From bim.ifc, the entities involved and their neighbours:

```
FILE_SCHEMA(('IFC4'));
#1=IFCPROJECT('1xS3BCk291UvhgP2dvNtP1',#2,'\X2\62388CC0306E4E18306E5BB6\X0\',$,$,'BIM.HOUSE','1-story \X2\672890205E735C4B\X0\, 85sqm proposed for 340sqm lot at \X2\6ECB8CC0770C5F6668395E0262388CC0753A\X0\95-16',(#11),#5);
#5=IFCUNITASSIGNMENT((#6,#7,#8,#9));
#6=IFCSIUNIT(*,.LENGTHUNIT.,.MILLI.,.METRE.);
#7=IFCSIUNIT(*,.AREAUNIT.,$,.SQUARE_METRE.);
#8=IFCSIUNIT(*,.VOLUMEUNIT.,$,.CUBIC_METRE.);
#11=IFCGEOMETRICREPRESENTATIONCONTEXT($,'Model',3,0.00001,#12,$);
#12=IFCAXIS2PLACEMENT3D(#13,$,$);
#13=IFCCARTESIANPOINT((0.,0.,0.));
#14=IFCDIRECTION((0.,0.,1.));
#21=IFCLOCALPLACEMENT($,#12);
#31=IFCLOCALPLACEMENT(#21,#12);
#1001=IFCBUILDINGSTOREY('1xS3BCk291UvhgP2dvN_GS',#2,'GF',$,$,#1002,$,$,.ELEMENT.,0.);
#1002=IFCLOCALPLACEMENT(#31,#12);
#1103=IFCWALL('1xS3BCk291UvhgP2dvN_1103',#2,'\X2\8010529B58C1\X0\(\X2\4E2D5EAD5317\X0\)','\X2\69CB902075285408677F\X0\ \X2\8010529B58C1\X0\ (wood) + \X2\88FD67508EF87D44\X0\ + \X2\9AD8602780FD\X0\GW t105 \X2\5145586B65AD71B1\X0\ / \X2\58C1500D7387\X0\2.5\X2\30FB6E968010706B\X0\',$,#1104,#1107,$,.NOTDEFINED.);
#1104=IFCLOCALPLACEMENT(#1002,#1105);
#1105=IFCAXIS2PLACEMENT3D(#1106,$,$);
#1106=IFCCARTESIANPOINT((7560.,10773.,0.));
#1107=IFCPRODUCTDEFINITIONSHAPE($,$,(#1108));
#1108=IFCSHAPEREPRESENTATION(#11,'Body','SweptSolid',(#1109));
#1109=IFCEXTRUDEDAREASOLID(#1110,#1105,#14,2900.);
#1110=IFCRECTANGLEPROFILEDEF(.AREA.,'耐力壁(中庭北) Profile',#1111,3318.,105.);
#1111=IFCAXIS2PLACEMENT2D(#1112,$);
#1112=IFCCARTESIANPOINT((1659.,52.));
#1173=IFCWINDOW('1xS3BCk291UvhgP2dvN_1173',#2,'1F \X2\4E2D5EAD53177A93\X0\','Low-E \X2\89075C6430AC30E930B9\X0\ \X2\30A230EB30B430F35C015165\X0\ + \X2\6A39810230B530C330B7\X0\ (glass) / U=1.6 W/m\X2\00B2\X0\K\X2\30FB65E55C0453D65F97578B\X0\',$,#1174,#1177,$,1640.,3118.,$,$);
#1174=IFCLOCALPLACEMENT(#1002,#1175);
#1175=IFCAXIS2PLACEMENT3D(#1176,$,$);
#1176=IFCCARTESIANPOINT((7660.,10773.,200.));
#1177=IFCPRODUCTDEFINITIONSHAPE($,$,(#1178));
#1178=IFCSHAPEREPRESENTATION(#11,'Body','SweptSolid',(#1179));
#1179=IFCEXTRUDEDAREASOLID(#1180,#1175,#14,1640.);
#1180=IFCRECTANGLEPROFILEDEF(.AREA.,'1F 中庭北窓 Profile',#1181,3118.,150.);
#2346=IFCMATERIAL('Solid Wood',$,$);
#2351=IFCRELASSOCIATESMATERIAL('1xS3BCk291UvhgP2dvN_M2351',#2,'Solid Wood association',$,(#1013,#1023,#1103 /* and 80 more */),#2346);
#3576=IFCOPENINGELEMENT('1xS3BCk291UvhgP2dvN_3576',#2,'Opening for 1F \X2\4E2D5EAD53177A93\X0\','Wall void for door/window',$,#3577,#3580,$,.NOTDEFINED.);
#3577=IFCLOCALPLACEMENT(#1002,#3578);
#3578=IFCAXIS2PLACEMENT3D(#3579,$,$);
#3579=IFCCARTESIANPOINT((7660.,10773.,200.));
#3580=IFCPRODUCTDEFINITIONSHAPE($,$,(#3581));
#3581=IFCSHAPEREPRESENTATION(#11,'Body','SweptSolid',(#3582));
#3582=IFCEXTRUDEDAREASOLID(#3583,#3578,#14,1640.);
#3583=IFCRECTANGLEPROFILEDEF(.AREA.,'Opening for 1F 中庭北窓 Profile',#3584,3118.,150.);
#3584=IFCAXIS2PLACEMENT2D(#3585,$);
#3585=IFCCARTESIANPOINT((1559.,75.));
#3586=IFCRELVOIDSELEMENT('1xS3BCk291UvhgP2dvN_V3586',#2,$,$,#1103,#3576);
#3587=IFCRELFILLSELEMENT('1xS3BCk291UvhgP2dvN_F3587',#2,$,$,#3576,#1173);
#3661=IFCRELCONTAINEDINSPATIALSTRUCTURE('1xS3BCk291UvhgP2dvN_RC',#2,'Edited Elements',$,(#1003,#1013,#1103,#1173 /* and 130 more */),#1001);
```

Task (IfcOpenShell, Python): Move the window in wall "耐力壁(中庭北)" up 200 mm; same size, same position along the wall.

```python
import numpy as np
import ifcopenshell
import ifcopenshell.api.geometry
import ifcopenshell.util.placement
import ifcopenshell.util.unit

model = ifcopenshell.open("bim.ifc")
unit_scale = ifcopenshell.util.unit.calculate_unit_scale(model)

window = model.by_id(1173)
opening = window.FillsVoids[0].RelatingOpeningElement
dz = 200.0

shift = np.array([0.0, 0.0, dz])
# The window is not placed relative to its opening, so move both.
for product in (opening, window):
    matrix = ifcopenshell.util.placement.get_local_placement(product.ObjectPlacement)
    matrix[:3, 3] += shift
    ifcopenshell.api.geometry.edit_object_placement(model, product=product, matrix=matrix, is_si=False)

print(f"moved by {dz * unit_scale:+.3f} m")

model.write("bim_updated.ifc")
```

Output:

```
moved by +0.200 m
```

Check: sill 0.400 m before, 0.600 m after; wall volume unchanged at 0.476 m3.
